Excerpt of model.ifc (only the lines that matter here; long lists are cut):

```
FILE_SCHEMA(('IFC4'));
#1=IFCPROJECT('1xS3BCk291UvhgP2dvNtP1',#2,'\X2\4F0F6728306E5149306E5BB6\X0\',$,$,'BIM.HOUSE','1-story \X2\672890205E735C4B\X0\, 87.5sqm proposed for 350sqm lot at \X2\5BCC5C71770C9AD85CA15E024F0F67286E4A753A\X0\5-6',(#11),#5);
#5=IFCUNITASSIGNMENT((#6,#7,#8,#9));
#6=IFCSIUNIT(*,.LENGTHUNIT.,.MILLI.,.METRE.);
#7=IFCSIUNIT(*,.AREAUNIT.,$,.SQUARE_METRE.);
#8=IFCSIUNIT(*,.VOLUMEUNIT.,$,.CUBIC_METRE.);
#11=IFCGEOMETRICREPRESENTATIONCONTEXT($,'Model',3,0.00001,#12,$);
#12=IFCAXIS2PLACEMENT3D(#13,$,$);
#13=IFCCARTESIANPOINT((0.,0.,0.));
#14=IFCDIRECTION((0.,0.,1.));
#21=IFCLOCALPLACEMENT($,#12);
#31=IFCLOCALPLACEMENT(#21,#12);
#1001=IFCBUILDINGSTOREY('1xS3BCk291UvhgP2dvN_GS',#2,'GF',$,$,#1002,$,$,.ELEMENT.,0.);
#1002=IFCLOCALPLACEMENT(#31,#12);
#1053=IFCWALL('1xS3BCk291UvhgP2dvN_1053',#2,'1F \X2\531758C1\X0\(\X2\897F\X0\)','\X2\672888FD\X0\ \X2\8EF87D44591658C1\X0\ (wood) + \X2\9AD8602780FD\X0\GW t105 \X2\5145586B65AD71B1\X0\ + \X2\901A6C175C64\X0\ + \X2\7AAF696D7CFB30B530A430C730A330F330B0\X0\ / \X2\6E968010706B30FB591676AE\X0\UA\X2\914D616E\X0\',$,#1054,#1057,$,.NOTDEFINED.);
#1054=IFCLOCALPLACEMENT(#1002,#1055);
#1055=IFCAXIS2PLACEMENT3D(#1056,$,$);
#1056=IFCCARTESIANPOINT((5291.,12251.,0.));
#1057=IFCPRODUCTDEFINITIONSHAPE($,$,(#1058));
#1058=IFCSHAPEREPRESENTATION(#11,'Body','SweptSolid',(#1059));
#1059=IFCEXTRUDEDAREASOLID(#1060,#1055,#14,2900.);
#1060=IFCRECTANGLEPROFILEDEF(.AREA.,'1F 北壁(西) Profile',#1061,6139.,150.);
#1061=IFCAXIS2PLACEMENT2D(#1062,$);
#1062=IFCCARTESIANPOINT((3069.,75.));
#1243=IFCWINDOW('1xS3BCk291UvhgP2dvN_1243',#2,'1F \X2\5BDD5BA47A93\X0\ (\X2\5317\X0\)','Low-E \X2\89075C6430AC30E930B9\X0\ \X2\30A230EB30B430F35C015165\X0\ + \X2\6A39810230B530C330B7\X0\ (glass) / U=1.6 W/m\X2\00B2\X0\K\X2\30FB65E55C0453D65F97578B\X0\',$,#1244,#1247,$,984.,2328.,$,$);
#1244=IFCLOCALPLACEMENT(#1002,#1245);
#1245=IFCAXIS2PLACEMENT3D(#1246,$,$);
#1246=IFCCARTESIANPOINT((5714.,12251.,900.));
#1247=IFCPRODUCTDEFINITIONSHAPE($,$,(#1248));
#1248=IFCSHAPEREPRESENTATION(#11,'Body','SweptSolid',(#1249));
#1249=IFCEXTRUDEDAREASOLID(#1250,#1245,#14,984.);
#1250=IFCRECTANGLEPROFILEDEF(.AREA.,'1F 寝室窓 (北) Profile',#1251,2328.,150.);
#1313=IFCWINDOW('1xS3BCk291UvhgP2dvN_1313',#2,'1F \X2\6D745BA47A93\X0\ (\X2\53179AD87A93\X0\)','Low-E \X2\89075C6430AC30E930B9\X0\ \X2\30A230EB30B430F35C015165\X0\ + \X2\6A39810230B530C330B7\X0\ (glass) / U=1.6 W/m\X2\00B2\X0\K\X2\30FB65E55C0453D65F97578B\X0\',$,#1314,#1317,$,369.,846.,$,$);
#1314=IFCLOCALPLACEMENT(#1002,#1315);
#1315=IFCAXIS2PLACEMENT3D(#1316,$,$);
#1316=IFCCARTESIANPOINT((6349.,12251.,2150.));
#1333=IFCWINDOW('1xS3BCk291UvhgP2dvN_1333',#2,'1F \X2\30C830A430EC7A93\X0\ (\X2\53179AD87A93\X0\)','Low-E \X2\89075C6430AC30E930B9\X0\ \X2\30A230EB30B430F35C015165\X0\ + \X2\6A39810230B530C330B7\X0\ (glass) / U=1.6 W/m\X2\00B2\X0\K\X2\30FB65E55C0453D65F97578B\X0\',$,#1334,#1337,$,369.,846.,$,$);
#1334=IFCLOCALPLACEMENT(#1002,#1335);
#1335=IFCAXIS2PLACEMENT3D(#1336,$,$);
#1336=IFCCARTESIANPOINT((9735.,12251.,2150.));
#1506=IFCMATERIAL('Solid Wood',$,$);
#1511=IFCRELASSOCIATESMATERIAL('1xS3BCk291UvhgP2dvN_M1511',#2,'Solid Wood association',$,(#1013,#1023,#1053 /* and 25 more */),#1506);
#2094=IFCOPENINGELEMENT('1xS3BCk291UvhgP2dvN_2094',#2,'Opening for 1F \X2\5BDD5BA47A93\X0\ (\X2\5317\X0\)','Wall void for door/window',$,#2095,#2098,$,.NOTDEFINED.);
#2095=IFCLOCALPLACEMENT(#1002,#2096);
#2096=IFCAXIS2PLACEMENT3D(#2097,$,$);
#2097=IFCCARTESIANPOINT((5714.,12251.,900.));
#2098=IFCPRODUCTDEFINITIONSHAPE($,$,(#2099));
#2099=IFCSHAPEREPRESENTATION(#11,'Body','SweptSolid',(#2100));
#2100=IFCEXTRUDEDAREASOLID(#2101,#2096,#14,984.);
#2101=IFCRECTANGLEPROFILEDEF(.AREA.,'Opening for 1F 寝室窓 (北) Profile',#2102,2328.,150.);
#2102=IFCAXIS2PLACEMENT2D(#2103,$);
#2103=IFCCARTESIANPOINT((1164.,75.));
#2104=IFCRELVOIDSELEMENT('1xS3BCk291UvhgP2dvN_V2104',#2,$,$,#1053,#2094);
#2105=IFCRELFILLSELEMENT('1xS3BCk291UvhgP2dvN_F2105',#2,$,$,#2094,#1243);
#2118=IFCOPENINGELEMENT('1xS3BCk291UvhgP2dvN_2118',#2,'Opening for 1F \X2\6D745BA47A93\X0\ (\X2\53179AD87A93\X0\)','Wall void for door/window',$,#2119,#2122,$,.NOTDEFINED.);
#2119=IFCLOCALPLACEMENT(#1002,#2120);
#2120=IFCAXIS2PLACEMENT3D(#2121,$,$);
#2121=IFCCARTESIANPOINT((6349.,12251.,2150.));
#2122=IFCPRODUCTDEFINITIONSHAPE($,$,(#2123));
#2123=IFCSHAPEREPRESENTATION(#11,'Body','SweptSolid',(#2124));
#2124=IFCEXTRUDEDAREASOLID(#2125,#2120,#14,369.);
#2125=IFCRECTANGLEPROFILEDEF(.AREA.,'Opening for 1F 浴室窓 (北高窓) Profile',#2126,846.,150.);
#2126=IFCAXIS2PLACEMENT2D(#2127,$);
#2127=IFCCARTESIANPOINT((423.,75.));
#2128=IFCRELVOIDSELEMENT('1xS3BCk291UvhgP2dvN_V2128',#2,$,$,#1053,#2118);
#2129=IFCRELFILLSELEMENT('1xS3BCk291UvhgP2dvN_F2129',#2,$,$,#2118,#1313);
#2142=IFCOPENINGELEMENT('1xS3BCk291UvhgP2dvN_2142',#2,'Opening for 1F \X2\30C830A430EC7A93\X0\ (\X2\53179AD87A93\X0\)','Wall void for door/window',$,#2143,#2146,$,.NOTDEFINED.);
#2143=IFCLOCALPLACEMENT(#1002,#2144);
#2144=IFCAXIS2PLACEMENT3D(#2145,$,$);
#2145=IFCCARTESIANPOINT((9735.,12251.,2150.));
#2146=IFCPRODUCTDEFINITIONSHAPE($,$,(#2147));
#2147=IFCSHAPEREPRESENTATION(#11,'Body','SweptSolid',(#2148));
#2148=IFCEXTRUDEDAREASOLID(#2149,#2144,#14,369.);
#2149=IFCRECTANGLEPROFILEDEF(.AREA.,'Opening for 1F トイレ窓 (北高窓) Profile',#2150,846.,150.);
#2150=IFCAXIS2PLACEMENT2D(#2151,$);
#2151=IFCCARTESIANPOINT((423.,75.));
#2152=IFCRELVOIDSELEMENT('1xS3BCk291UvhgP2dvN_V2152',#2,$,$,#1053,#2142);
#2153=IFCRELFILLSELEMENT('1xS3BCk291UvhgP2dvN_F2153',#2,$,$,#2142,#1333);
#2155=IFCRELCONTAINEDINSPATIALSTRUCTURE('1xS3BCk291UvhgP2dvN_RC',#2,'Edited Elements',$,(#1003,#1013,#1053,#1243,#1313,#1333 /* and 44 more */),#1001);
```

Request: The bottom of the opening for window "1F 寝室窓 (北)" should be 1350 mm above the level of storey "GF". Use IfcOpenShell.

```python
import numpy as np
import ifcopenshell
import ifcopenshell.api.geometry
import ifcopenshell.geom
import ifcopenshell.util.element
import ifcopenshell.util.placement
import ifcopenshell.util.shape
import ifcopenshell.util.unit

model = ifcopenshell.open("model.ifc")
unit_scale = ifcopenshell.util.unit.calculate_unit_scale(model)

window = model.by_guid("1xS3BCk291UvhgP2dvN_1243")
opening = window.FillsVoids[0].RelatingOpeningElement
storey = ifcopenshell.util.element.get_container(window, ifc_class="IfcBuildingStorey")
level = ifcopenshell.util.placement.get_local_placement(storey.ObjectPlacement)[2, 3]

# The opening's origin need not be at the sill, so measure its lowest point.
shape = ifcopenshell.geom.create_shape(ifcopenshell.geom.settings(), opening)
bottom = ifcopenshell.util.shape.get_shape_bottom_elevation(shape, shape.geometry) / unit_scale
dz = level + 1.35 / unit_scale - bottom

shift = np.array([0.0, 0.0, dz])
# The window is not placed relative to its opening, so move both.
for product in (opening, window):
    matrix = ifcopenshell.util.placement.get_local_placement(product.ObjectPlacement)
    matrix[:3, 3] += shift
    ifcopenshell.api.geometry.edit_object_placement(model, product=product, matrix=matrix, is_si=False)

print(f"moved by {dz * unit_scale:+.3f} m")

model.write("model_updated.ifc")
```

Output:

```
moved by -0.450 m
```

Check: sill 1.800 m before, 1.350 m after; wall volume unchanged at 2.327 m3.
